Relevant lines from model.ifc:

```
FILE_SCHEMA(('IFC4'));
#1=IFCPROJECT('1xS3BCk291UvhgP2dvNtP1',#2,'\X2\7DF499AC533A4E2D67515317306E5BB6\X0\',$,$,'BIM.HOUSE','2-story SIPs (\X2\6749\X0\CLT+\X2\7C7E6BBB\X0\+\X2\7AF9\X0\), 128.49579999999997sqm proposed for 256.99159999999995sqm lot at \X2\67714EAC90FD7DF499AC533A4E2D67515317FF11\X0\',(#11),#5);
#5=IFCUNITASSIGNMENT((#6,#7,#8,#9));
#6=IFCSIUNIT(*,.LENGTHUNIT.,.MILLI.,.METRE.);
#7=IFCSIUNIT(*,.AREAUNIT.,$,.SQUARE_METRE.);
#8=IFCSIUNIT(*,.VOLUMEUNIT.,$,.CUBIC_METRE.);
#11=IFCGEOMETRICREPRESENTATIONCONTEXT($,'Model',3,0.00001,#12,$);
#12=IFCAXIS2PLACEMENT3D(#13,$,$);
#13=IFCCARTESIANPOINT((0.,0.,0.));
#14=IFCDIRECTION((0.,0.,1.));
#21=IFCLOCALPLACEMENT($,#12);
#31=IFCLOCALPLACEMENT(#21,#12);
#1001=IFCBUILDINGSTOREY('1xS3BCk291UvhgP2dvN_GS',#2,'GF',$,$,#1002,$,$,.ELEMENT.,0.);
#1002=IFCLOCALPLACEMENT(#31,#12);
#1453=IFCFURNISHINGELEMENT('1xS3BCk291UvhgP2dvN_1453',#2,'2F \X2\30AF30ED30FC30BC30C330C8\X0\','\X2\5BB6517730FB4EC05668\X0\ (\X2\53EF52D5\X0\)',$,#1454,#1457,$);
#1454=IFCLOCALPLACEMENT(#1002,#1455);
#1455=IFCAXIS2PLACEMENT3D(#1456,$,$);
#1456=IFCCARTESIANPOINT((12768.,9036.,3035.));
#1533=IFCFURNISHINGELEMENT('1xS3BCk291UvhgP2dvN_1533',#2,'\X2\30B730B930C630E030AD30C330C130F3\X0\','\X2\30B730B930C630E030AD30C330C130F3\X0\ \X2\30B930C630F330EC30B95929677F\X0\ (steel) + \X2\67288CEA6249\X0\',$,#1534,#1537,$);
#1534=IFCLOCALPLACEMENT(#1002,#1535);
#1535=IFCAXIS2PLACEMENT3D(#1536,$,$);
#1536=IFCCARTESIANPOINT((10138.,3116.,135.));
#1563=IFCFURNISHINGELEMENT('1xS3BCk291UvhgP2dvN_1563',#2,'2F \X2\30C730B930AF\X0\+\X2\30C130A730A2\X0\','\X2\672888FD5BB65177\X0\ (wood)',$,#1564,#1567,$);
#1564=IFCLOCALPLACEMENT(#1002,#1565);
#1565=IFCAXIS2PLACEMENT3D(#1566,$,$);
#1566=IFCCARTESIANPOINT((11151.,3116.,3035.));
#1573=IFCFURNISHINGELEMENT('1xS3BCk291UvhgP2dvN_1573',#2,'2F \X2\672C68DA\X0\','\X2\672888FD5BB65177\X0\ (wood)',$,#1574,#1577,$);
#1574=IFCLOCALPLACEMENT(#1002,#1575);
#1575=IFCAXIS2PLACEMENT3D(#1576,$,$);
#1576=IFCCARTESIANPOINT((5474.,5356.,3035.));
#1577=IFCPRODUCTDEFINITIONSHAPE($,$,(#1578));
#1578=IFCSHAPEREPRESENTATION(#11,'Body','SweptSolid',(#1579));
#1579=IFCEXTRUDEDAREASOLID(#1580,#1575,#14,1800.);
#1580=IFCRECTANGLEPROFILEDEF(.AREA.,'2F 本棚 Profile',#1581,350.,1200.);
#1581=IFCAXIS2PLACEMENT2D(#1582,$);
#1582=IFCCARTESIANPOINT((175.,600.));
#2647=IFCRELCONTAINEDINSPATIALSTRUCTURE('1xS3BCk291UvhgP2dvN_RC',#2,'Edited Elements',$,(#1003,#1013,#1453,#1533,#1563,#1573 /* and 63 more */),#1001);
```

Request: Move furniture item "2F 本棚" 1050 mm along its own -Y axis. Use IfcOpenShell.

```python
import ifcopenshell
import ifcopenshell.api.geometry
import ifcopenshell.util.placement
import ifcopenshell.util.unit

model = ifcopenshell.open("model.ifc")
unit_scale = ifcopenshell.util.unit.calculate_unit_scale(model)

item = model.by_id(1573)
matrix = ifcopenshell.util.placement.get_local_placement(item.ObjectPlacement)
matrix[:3, 3] -= matrix[:3, 1] * 1.05 / unit_scale
ifcopenshell.api.geometry.edit_object_placement(model, product=item, matrix=matrix, is_si=False)

print(ifcopenshell.util.placement.get_local_placement(item.ObjectPlacement).round(3) + 0.0)

model.write("model_edited.ifc")
```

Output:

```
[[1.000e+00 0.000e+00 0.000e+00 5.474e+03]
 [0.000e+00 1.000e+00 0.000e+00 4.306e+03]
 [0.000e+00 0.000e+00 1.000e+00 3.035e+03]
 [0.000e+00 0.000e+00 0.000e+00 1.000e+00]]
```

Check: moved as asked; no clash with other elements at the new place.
